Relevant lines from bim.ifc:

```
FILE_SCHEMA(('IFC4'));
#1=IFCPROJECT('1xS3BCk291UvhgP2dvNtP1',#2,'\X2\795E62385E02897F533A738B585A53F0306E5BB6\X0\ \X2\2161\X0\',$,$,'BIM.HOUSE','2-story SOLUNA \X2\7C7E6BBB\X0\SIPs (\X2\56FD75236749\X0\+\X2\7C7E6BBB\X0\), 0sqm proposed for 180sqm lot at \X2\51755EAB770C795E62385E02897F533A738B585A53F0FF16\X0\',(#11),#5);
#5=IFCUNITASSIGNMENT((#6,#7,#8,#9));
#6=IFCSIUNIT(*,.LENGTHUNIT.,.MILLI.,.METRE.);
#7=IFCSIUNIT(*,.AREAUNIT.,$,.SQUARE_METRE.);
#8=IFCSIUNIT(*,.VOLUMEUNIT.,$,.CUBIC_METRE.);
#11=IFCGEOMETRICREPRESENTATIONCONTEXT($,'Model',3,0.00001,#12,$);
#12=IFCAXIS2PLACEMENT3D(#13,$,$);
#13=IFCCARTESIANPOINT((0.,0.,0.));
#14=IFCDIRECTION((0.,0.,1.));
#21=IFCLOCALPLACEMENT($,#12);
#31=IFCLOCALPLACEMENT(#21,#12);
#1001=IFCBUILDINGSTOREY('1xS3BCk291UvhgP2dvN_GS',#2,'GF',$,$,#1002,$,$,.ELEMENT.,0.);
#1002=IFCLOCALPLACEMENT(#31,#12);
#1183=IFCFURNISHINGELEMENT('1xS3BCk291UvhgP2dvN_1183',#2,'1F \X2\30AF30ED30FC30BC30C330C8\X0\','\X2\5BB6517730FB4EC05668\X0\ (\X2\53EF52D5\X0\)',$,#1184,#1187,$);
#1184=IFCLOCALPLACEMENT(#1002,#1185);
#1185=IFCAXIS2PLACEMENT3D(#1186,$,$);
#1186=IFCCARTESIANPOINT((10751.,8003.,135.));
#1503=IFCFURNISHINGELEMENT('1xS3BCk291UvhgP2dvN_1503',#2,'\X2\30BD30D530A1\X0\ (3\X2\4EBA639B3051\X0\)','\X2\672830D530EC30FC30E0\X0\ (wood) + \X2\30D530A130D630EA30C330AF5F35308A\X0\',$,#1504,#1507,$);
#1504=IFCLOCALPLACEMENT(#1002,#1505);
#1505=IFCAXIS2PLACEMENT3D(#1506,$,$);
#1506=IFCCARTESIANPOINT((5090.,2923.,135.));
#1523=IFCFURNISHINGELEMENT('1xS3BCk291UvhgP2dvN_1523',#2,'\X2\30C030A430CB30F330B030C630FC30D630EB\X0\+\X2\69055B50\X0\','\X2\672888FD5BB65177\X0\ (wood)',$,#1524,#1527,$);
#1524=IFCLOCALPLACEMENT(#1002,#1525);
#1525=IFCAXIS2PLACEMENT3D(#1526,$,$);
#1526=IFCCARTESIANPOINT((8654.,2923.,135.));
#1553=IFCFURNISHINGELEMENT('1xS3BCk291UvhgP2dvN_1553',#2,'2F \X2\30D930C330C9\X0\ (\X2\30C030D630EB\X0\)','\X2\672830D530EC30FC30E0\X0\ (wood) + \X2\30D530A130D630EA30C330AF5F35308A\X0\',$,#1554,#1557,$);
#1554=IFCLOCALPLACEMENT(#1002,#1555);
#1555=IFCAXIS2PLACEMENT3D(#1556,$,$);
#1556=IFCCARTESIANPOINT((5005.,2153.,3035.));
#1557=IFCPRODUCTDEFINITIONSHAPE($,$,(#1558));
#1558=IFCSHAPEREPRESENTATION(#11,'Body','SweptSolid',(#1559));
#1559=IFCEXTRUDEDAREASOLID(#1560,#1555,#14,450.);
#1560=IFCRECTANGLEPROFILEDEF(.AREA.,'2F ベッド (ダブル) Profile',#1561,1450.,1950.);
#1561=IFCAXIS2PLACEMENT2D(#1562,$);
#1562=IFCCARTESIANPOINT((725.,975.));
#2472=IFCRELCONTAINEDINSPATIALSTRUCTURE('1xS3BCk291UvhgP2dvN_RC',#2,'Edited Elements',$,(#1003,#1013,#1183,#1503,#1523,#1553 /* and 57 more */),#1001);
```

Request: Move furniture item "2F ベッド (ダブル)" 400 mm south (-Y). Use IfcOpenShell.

```python
import ifcopenshell
import ifcopenshell.api.geometry
import ifcopenshell.util.placement
import ifcopenshell.util.unit

model = ifcopenshell.open("bim.ifc")
unit_scale = ifcopenshell.util.unit.calculate_unit_scale(model)

item = model.by_guid("1xS3BCk291UvhgP2dvN_1553")
matrix = ifcopenshell.util.placement.get_local_placement(item.ObjectPlacement)
matrix[1, 3] -= 0.4 / unit_scale
ifcopenshell.api.geometry.edit_object_placement(model, product=item, matrix=matrix, is_si=False)

print(ifcopenshell.util.placement.get_local_placement(item.ObjectPlacement).round(3) + 0.0)

model.write("bim_edited.ifc")
```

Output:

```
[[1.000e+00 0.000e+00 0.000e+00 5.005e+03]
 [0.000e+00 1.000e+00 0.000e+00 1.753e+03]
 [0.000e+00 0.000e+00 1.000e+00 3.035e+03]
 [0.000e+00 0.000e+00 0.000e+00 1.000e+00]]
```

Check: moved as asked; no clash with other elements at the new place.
